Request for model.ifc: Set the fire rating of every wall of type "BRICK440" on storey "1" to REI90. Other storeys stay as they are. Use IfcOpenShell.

First a look at what the model holds.

```python
import ifcopenshell
import ifcopenshell.util.element

model = ifcopenshell.open("model.ifc")
print(model.schema)
storey = next(s for s in model.by_type("IfcBuildingStorey") if s.Name == "1")
walls = [e for e in ifcopenshell.util.element.get_decomposition(storey) if e.is_a("IfcWall")]
seen = {}
for e in walls:
    element_type = ifcopenshell.util.element.get_type(e)
    key = (element_type.Name if element_type != e and element_type else None, ifcopenshell.util.element.get_pset(e, "Pset_WallCommon", "FireRating"))
    seen[key] = seen.get(key, 0) + 1
for (name, value), count in sorted(seen.items(), key=str):
    print(count, "x", name, "|", value)
```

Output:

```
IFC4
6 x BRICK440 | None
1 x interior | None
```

```python
import ifcopenshell
import ifcopenshell.api.pset
import ifcopenshell.util.element

model = ifcopenshell.open("model.ifc")

storey = next(s for s in model.by_type("IfcBuildingStorey") if s.Name == "1")
walls = [e for e in ifcopenshell.util.element.get_decomposition(storey) if e.is_a("IfcWall")]

count = 0
for e in walls:
    element_type = ifcopenshell.util.element.get_type(e)
    if element_type in (None, e) or element_type.Name != "BRICK440":
        continue
    # add_pset returns the element's existing set when there is one.
    pset = ifcopenshell.api.pset.add_pset(model, product=e, name="Pset_WallCommon")
    ifcopenshell.api.pset.edit_pset(model, pset=pset, properties={"FireRating": "REI90"})
    count += 1

print(count, "walls updated")

model.write("model_edited.ifc")
```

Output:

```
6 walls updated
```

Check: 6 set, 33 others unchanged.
